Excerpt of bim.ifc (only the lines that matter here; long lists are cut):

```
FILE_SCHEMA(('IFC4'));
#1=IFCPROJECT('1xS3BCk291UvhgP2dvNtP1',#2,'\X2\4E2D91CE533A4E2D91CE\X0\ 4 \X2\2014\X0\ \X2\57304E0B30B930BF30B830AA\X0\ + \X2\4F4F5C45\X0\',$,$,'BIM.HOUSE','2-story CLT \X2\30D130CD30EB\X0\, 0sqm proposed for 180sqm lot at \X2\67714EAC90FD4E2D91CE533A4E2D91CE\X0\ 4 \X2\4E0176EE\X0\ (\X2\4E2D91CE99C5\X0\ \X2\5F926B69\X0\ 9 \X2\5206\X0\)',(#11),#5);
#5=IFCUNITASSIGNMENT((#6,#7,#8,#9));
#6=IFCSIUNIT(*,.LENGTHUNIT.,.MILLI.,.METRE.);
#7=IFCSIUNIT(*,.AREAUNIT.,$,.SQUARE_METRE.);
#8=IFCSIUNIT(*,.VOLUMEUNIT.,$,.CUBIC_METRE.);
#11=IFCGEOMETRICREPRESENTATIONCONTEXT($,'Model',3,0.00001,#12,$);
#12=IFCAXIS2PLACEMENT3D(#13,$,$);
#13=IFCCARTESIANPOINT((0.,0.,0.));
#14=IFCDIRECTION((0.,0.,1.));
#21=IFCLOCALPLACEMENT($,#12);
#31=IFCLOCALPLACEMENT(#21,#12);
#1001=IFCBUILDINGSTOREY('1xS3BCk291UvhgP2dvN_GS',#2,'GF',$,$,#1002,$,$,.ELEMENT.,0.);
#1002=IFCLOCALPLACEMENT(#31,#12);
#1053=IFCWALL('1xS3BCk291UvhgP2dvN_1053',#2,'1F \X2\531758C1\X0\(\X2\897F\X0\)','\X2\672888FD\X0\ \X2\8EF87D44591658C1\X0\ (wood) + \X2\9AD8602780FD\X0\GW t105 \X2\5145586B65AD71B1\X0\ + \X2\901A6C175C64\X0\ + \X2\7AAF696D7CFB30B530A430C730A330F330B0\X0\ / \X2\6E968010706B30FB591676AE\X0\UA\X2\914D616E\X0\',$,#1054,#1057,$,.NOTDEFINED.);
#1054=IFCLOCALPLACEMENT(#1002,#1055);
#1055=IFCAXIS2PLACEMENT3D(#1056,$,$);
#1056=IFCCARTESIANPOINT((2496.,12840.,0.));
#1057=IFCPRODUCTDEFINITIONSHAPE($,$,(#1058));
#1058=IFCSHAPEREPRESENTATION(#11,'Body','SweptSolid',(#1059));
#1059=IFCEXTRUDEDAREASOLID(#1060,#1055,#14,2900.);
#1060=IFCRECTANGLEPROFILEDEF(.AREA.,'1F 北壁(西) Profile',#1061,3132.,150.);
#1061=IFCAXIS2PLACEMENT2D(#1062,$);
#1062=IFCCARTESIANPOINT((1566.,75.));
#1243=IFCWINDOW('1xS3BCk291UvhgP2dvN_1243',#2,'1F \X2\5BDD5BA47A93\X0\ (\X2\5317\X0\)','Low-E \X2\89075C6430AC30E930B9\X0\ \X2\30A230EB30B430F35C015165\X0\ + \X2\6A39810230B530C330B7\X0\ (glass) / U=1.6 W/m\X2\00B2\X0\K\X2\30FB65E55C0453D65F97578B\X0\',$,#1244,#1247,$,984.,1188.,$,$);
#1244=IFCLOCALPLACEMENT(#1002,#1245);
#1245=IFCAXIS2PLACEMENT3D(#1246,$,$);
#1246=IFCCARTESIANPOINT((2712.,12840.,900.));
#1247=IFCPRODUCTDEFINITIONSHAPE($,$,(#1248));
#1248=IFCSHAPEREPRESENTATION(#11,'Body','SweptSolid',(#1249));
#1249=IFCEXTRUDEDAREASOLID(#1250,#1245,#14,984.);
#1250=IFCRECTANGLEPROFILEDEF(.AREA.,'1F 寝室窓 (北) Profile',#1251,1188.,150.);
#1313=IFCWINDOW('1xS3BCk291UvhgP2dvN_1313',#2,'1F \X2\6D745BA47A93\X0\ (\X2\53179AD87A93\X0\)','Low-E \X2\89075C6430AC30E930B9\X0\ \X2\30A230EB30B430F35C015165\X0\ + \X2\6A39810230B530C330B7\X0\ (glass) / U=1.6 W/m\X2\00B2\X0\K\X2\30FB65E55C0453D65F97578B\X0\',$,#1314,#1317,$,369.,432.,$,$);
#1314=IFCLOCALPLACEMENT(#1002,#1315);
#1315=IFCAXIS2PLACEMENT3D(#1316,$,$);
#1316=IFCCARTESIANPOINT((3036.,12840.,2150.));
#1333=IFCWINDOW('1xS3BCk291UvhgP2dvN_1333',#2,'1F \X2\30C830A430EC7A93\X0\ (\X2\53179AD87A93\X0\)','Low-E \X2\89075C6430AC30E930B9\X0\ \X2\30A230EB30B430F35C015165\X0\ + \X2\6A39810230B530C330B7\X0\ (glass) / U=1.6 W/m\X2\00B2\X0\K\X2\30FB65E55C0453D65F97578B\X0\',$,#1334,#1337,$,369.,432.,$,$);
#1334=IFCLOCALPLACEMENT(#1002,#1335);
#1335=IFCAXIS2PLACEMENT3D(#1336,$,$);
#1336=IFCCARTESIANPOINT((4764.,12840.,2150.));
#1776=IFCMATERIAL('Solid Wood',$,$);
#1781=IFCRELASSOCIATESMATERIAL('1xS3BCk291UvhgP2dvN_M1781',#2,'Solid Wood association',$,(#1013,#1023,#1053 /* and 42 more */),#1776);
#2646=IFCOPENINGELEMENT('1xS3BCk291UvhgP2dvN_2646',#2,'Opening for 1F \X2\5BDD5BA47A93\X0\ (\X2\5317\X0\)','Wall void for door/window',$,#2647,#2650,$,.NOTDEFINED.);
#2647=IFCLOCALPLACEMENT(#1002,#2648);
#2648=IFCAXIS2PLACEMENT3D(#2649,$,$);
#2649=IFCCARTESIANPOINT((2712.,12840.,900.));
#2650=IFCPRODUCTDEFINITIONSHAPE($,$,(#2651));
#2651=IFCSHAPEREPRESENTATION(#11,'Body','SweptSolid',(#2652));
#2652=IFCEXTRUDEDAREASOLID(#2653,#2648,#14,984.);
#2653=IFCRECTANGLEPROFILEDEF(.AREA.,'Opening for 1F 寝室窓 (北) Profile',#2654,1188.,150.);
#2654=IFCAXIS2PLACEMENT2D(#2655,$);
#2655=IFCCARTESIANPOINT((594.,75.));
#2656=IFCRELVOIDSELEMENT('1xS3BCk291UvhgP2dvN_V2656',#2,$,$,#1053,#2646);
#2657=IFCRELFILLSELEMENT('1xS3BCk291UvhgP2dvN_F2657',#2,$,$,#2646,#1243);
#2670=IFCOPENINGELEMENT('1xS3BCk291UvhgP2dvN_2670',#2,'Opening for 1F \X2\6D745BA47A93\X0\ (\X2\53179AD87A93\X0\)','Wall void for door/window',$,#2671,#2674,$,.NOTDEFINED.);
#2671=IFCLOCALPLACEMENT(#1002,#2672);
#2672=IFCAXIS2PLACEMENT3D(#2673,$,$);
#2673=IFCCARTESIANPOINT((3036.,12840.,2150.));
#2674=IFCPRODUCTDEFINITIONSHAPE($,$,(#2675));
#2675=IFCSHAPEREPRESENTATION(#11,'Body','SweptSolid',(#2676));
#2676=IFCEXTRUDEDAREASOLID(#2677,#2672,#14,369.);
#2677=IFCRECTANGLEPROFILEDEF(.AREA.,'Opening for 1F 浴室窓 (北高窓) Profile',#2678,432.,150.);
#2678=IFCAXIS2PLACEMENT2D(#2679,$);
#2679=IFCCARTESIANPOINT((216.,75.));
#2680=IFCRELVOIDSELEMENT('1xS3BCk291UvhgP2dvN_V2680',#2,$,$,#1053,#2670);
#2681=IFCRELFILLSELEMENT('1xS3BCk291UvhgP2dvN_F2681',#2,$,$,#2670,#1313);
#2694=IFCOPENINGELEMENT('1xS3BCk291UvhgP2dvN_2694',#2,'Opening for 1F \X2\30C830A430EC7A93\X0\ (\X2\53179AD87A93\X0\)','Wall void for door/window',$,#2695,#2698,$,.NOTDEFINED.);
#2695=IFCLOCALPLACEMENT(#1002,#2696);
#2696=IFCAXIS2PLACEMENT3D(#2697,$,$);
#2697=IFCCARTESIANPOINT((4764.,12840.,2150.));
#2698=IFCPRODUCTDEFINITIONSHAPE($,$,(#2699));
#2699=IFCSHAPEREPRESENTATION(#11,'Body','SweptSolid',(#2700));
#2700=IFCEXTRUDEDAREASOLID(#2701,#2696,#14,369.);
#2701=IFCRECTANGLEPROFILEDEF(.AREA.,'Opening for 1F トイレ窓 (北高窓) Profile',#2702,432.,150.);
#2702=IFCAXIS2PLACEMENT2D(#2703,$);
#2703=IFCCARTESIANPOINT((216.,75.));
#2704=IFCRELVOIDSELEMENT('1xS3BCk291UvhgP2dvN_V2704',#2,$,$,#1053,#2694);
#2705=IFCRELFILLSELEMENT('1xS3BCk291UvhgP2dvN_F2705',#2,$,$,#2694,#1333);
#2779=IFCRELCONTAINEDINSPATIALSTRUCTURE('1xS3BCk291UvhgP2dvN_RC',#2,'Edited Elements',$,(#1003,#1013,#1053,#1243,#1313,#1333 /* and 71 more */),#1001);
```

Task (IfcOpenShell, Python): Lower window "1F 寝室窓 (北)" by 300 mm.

```python
import numpy as np
import ifcopenshell
import ifcopenshell.api.geometry
import ifcopenshell.util.placement
import ifcopenshell.util.unit

model = ifcopenshell.open("bim.ifc")
unit_scale = ifcopenshell.util.unit.calculate_unit_scale(model)

window = model.by_guid("1xS3BCk291UvhgP2dvN_1243")
opening = window.FillsVoids[0].RelatingOpeningElement
dz = -0.3 / unit_scale

shift = np.array([0.0, 0.0, dz])
# The window is not placed relative to its opening, so move both.
for product in (opening, window):
    matrix = ifcopenshell.util.placement.get_local_placement(product.ObjectPlacement)
    matrix[:3, 3] += shift
    ifcopenshell.api.geometry.edit_object_placement(model, product=product, matrix=matrix, is_si=False)

print(f"moved by {dz * unit_scale:+.3f} m")

model.write("bim_edited.ifc")
```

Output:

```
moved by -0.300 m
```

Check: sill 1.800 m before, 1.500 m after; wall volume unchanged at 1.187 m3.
